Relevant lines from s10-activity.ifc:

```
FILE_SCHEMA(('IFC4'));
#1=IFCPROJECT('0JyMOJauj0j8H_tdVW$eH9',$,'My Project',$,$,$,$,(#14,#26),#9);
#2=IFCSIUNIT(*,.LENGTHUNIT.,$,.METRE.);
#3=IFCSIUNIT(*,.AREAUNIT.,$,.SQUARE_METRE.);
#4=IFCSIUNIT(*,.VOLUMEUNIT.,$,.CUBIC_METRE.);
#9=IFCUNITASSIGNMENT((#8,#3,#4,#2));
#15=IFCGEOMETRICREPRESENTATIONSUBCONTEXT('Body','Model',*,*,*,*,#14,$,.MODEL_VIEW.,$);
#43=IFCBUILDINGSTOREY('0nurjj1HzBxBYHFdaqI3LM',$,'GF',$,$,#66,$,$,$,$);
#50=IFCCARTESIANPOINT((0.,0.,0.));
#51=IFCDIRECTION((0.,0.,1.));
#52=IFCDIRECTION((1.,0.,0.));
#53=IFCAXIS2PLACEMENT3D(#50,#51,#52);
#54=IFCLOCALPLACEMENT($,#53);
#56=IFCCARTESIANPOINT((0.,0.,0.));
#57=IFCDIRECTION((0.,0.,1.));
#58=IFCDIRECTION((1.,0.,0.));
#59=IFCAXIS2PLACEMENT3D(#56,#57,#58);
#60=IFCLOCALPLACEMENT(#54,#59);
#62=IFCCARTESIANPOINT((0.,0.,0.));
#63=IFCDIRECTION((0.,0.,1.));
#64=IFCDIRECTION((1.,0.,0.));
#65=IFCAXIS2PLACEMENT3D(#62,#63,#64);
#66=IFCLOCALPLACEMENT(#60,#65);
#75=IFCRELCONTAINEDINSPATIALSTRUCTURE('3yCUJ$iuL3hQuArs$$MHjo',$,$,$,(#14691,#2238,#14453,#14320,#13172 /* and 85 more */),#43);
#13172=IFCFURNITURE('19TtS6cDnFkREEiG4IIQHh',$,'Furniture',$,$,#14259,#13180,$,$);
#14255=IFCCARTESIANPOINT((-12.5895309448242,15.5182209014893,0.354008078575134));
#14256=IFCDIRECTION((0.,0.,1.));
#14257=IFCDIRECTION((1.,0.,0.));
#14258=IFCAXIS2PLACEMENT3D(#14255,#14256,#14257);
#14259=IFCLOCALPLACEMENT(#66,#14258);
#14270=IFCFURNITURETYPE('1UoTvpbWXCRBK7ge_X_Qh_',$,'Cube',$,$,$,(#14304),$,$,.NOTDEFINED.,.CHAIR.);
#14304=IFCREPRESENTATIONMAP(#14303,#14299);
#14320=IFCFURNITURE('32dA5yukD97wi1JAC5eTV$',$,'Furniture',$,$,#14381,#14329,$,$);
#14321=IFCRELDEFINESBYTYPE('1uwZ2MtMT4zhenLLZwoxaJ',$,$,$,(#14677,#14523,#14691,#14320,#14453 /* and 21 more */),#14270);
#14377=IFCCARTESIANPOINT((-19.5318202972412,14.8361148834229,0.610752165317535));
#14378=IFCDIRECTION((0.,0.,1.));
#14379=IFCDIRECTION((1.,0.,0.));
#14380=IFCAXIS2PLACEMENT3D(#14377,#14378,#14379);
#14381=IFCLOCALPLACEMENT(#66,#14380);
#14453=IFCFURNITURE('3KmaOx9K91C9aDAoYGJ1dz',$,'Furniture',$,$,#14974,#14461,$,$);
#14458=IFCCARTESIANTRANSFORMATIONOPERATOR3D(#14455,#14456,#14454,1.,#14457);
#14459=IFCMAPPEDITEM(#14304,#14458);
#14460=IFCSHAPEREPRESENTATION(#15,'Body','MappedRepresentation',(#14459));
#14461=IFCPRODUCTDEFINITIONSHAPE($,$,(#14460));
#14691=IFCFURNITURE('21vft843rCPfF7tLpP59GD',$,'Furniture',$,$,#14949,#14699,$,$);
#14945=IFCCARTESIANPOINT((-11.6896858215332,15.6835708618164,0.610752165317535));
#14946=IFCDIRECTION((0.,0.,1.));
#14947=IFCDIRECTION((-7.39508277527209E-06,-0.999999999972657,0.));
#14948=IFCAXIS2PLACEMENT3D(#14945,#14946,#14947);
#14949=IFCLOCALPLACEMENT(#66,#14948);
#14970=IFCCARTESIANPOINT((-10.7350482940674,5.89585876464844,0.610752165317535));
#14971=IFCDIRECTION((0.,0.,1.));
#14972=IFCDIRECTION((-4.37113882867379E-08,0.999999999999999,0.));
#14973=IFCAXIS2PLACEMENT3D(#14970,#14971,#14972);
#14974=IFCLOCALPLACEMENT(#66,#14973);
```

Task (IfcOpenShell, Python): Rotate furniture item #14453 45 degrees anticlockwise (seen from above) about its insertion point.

```python
import ifcopenshell
import ifcopenshell.api.geometry
import ifcopenshell.util.placement

model = ifcopenshell.open("s10-activity.ifc")

item = model.by_id(14453)
matrix = ifcopenshell.util.placement.get_local_placement(item.ObjectPlacement)
matrix = matrix @ ifcopenshell.util.placement.rotation(45, "Z")
ifcopenshell.api.geometry.edit_object_placement(model, product=item, matrix=matrix, is_si=False)

print(ifcopenshell.util.placement.get_local_placement(item.ObjectPlacement).round(3) + 0.0)

model.write("s10-activity_rev.ifc")
```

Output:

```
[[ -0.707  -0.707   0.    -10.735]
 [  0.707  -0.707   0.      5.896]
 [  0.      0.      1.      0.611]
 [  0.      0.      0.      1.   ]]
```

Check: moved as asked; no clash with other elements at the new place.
